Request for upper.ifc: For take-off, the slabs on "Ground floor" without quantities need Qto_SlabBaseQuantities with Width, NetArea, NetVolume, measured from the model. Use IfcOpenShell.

First a look at what the model holds.

```python
import ifcopenshell
import ifcopenshell.util.element
import ifcopenshell.util.unit

model = ifcopenshell.open("upper.ifc")
print(model.schema)
for unit_type in ("LENGTHUNIT", "AREAUNIT", "VOLUMEUNIT"):
    print(unit_type, ifcopenshell.util.unit.calculate_unit_scale(model, unit_type))
storey = next(s for s in model.by_type("IfcBuildingStorey") if s.Name == "Ground floor")
slabs = [e for e in ifcopenshell.util.element.get_decomposition(storey) if e.is_a("IfcSlab")]
for e in sorted(slabs, key=lambda e: e.id()):
    print(e.id(), e.is_a(), e.Name, list(ifcopenshell.util.element.get_psets(e, qtos_only=True)), sep=" | ")
```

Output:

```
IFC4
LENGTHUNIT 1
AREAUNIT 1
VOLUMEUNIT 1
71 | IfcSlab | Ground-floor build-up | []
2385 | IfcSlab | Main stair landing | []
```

```python
import ifcopenshell
import ifcopenshell.api.pset
import ifcopenshell.geom
import ifcopenshell.util.element
import ifcopenshell.util.shape
import ifcopenshell.util.unit

model = ifcopenshell.open("upper.ifc")
unit_scale = ifcopenshell.util.unit.calculate_unit_scale(model)
area_scale = ifcopenshell.util.unit.calculate_unit_scale(model, "AREAUNIT")
volume_scale = ifcopenshell.util.unit.calculate_unit_scale(model, "VOLUMEUNIT")
settings = ifcopenshell.geom.settings()

storey = next(s for s in model.by_type("IfcBuildingStorey") if s.Name == "Ground floor")
slabs = [e for e in ifcopenshell.util.element.get_decomposition(storey) if e.is_a("IfcSlab")]

for e in sorted(slabs, key=lambda e: e.id()):
    if ifcopenshell.util.element.get_psets(e, qtos_only=True, should_inherit=False):
        continue
    # Geometry comes back in metres, in the element's own axes.
    shape = ifcopenshell.geom.create_shape(settings, e)
    values = {
        "Width": ifcopenshell.util.shape.get_z(shape.geometry) / unit_scale,
        "NetArea": ifcopenshell.util.shape.get_footprint_area(shape.geometry) / area_scale,
        "NetVolume": ifcopenshell.util.shape.get_volume(shape.geometry) / volume_scale,
    }
    qto = ifcopenshell.api.pset.add_qto(model, product=e, name="Qto_SlabBaseQuantities")
    ifcopenshell.api.pset.edit_qto(model, qto=qto, properties=values)
    print(e.id(), {k: round(v, 3) for k, v in values.items()})

model.write("upper_rev.ifc")
```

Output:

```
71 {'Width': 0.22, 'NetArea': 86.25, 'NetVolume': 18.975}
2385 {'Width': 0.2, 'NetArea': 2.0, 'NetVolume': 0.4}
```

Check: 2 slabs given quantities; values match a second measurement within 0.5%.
